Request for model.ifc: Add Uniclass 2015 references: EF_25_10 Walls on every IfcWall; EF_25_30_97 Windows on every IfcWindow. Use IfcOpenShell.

First a look at what the model holds.

```python
import ifcopenshell

model = ifcopenshell.open("model.ifc")
print(model.schema)
print("classifications:", [c.Name for c in model.by_type("IfcClassification")])
for ifc_class in ("IfcDoor", "IfcRoof", "IfcStair", "IfcWall", "IfcWindow"):
    print(ifc_class, len(model.by_type(ifc_class)))
```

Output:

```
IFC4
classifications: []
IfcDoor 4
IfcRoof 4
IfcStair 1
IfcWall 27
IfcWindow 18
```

```python
import ifcopenshell
import ifcopenshell.api.classification

model = ifcopenshell.open("model.ifc")

system = ifcopenshell.api.classification.add_classification(model, classification="Uniclass 2015")

codes = {
    "IfcWall": ("EF_25_10", "Walls"),
    "IfcWindow": ("EF_25_30_97", "Windows"),
}
for ifc_class, (code, name) in codes.items():
    products = model.by_type(ifc_class)
    ifcopenshell.api.classification.add_reference(
        model, products=products, classification=system, identification=code, name=name
    )
    print(code, len(products))

model.write("model-out.ifc")
```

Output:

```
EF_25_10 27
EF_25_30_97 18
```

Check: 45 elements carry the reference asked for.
